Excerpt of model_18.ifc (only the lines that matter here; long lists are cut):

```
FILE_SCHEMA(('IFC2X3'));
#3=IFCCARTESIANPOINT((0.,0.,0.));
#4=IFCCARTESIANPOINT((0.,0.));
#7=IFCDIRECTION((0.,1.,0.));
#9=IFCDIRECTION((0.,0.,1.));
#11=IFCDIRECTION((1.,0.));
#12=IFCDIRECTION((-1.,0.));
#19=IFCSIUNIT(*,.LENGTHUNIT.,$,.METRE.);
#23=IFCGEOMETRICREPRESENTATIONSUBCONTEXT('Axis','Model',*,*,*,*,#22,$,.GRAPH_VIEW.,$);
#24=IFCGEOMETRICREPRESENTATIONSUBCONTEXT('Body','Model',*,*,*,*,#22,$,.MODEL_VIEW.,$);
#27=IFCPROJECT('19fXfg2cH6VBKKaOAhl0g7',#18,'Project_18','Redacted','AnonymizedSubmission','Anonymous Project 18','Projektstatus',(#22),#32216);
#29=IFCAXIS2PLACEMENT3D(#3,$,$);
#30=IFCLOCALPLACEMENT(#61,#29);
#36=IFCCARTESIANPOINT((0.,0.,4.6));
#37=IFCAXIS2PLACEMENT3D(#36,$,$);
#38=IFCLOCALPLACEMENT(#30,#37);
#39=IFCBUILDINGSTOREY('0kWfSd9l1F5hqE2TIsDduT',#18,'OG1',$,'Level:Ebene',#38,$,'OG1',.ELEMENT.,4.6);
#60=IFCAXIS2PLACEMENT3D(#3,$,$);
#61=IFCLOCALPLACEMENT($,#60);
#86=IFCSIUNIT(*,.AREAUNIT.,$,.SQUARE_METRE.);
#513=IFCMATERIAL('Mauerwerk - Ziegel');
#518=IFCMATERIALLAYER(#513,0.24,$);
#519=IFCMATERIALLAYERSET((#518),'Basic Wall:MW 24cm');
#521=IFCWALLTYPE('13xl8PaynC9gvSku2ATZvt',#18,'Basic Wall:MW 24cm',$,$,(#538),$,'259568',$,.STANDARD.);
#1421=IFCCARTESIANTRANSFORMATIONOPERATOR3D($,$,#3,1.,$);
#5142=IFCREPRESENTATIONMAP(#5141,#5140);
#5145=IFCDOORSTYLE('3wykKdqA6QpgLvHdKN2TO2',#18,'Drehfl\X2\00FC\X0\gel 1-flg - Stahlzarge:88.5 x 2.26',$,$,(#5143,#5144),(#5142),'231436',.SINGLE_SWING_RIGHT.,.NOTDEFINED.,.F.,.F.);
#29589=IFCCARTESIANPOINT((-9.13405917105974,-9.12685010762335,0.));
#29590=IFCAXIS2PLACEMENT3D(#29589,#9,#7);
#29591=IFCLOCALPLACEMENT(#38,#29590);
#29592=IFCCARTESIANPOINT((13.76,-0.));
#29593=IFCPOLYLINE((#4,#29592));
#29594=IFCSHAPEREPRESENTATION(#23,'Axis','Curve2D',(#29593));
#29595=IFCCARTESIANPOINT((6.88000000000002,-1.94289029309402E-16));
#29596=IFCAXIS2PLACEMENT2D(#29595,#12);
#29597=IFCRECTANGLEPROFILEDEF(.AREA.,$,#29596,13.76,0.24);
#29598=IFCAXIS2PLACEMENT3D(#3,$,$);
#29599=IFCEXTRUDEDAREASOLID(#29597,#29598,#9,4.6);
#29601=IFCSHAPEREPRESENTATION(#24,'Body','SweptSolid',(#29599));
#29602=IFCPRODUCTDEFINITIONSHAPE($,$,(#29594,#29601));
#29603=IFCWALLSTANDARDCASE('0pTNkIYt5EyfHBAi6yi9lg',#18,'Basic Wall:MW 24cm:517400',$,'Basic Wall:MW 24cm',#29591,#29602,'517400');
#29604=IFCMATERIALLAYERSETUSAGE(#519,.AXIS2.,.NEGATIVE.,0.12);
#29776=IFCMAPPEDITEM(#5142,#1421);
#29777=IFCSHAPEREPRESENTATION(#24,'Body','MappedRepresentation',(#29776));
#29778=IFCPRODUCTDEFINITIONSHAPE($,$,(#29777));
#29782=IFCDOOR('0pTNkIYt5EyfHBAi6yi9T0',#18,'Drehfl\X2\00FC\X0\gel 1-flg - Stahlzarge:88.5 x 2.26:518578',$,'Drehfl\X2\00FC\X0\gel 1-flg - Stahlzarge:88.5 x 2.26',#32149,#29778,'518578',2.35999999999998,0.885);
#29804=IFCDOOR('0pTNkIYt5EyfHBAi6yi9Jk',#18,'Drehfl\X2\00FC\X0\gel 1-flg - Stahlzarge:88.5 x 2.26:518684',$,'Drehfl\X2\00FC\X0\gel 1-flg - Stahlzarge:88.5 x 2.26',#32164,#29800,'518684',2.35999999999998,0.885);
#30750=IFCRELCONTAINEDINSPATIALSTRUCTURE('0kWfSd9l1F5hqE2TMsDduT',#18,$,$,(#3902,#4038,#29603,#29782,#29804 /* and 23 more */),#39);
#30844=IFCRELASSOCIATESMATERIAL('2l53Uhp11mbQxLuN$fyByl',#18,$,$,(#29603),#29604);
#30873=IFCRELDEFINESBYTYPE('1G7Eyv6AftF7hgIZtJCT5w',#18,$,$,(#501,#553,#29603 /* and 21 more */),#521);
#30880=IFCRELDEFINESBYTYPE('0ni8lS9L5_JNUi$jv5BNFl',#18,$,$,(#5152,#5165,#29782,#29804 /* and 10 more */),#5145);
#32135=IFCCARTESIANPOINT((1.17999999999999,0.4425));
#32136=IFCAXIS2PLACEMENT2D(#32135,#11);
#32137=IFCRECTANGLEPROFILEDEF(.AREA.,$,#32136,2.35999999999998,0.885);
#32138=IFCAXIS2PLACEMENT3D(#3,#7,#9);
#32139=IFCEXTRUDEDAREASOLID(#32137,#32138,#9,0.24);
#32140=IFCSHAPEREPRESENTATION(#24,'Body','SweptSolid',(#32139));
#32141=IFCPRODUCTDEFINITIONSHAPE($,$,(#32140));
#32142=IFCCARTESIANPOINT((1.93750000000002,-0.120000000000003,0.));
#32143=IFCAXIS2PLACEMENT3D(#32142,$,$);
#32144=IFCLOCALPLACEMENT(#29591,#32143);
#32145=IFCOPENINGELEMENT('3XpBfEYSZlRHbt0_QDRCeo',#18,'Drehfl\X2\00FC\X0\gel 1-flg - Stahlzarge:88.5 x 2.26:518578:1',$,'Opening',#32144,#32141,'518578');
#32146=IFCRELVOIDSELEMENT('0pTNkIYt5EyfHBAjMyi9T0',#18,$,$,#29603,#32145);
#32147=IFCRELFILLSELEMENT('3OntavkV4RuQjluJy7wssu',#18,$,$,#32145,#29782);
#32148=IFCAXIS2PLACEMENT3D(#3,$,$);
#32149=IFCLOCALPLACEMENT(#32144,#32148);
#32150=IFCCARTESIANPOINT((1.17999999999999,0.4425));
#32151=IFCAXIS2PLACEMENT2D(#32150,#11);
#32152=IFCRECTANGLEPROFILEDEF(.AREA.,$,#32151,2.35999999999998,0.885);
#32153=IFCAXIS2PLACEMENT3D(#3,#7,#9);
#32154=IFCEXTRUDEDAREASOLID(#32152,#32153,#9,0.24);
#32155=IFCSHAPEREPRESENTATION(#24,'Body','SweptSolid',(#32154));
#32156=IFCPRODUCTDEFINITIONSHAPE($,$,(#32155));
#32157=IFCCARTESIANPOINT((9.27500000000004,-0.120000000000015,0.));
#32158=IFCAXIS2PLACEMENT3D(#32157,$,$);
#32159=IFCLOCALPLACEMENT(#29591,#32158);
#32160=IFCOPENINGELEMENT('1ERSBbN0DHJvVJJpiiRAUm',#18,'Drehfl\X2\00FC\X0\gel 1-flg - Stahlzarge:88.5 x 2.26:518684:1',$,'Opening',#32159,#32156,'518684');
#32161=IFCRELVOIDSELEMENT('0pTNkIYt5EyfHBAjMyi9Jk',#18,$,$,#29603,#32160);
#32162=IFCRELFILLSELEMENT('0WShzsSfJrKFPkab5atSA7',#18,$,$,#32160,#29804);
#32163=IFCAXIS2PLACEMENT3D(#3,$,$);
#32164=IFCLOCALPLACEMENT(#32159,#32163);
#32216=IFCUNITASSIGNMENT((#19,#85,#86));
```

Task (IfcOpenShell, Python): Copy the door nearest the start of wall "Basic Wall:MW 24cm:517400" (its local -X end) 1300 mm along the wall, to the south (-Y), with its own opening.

```python
import ifcopenshell
import ifcopenshell.api.feature
import ifcopenshell.api.geometry
import ifcopenshell.api.root
import ifcopenshell.geom
import ifcopenshell.util.element
import ifcopenshell.util.placement
import ifcopenshell.util.shape
import ifcopenshell.util.unit

model = ifcopenshell.open("model_18.ifc")
unit_scale = ifcopenshell.util.unit.calculate_unit_scale(model)
settings = ifcopenshell.geom.settings()


def volume(element):
    """Net volume in cubic metres, openings subtracted."""
    shape = ifcopenshell.geom.create_shape(settings, element)
    return ifcopenshell.util.shape.get_volume(shape.geometry)


def reuse_history(source, copy):
    """copy_class also copies each property set's owner history, people and application; keep the originals."""
    for rel in copy.IsDefinedBy:
        if rel.is_a("IfcRelDefinesByProperties") and (history := rel.RelatingPropertyDefinition.OwnerHistory):
            rel.RelatingPropertyDefinition.OwnerHistory = source.OwnerHistory
            ifcopenshell.util.element.remove_deep2(model, history)


door = model.by_guid("0pTNkIYt5EyfHBAi6yi9T0")
opening = door.FillsVoids[0].RelatingOpeningElement
wall = opening.VoidsElements[0].RelatingBuildingElement
before = volume(wall)
shift = ifcopenshell.util.placement.get_local_placement(wall.ObjectPlacement)[:3, 0] * -1.3 / unit_scale

# copy_class copies the void relationship, type, container and properties, but no geometry.
new_opening = ifcopenshell.api.root.copy_class(model, product=opening)
new_opening.Representation = ifcopenshell.util.element.copy_deep(
    model, opening.Representation, exclude=["IfcGeometricRepresentationContext", "IfcRepresentationMap"]
)
new_opening.Name = "Drehflügel 1-flg - Stahlzarge:88.5 x 2.26"
new_opening.Tag = None
new_door = ifcopenshell.api.root.copy_class(model, product=door)
new_door.Representation = ifcopenshell.util.element.copy_deep(
    model, door.Representation, exclude=["IfcGeometricRepresentationContext", "IfcRepresentationMap"]
)
new_door.Name = "Drehflügel 1-flg - Stahlzarge:88.5 x 2.26"
new_door.Tag = None
reuse_history(door, new_door)
fills = ifcopenshell.api.feature.add_filling(model, opening=new_opening, element=new_door)
fills.OwnerHistory = new_door.OwnerHistory  # required in IFC2X3

for old, new in ((opening, new_opening), (door, new_door)):
    matrix = ifcopenshell.util.placement.get_local_placement(old.ObjectPlacement)
    matrix[:3, 3] += shift
    ifcopenshell.api.geometry.edit_object_placement(model, product=new, matrix=matrix, is_si=False)

after = volume(wall)

print(f"wall volume {before:.3f} -> {after:.3f} m3")

model.write("model_18_updated.ifc")
```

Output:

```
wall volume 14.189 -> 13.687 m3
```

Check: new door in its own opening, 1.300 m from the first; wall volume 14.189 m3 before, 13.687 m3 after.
